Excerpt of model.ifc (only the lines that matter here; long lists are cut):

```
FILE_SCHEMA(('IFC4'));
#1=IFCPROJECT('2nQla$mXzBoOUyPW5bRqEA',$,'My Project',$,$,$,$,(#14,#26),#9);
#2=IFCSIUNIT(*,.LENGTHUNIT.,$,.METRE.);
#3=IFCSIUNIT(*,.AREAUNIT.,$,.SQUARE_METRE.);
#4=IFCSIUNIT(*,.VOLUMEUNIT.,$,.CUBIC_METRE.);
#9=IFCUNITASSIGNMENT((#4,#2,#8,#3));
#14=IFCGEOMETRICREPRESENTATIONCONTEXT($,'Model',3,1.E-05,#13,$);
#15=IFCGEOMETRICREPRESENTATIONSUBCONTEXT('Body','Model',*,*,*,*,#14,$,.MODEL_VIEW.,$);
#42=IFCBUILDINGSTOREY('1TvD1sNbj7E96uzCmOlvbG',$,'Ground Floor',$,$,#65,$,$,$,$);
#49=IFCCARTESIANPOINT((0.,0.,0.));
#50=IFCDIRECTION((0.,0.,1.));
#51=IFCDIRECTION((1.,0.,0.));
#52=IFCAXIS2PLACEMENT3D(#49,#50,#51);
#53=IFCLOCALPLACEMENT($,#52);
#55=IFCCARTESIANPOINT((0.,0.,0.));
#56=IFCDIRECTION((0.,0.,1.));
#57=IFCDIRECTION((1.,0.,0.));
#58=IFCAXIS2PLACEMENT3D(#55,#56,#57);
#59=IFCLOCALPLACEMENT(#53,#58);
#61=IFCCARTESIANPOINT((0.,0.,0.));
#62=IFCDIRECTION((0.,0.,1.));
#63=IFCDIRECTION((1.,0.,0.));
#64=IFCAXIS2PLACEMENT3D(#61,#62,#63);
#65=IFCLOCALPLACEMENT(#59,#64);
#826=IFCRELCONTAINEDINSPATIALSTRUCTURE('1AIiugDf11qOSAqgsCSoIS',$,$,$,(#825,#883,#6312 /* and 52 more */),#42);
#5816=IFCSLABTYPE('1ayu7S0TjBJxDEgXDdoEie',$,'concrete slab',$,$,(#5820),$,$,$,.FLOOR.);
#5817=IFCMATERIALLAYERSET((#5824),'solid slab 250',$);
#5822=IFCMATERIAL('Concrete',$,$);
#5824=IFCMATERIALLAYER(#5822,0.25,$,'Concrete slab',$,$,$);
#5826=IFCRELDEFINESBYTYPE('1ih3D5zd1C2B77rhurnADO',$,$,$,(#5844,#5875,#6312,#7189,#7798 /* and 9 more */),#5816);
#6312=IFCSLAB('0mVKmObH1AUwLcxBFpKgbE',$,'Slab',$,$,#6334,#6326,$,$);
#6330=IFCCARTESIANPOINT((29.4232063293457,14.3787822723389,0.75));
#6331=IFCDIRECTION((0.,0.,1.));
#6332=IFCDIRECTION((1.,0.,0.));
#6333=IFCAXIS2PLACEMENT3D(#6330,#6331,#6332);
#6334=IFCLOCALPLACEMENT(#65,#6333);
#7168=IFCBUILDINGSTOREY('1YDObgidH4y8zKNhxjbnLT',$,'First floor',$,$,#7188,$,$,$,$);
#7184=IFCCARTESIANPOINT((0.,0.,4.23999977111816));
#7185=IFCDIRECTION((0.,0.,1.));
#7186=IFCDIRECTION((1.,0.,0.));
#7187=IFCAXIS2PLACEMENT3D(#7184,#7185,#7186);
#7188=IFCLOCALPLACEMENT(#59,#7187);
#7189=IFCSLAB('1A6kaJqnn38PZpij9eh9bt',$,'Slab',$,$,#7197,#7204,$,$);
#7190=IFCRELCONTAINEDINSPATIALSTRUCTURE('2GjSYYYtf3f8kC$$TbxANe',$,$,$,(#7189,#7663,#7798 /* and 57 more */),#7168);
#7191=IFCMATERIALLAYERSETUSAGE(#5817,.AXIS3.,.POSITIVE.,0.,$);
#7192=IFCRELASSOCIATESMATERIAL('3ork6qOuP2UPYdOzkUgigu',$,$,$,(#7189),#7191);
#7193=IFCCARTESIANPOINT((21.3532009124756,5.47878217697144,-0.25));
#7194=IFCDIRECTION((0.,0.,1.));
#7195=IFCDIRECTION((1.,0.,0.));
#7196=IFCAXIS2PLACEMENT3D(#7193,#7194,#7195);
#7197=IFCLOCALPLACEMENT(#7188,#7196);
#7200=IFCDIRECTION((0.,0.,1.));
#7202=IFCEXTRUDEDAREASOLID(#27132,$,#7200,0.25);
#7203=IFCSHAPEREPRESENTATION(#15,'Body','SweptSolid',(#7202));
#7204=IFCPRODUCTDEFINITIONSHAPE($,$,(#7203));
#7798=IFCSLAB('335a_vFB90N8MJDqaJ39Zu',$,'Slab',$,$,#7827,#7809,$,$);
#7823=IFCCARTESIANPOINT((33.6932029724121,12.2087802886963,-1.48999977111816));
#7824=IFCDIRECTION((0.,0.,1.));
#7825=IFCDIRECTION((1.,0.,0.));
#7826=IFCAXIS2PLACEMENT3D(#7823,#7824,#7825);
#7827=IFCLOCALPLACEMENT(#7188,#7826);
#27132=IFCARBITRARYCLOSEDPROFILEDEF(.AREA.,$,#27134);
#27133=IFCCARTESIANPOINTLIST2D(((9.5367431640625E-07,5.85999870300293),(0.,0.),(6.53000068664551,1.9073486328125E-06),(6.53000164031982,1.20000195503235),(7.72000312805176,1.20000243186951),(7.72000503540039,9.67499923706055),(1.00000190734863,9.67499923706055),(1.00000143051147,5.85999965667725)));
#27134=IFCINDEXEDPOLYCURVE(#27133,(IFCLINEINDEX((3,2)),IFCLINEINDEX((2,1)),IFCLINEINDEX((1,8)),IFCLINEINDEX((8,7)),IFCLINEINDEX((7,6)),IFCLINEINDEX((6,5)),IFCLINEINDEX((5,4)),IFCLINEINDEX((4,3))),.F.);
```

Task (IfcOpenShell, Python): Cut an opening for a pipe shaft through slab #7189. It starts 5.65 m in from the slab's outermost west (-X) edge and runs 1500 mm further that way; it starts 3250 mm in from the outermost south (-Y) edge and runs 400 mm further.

```python
import numpy as np
import ifcopenshell
import ifcopenshell.api.feature
import ifcopenshell.api.geometry
import ifcopenshell.api.root
import ifcopenshell.geom
import ifcopenshell.util.placement
import ifcopenshell.util.representation
import ifcopenshell.util.shape
import ifcopenshell.util.unit

model = ifcopenshell.open("model.ifc")
unit_scale = ifcopenshell.util.unit.calculate_unit_scale(model)
settings = ifcopenshell.geom.settings()


def volume(element):
    """Net volume in cubic metres, openings subtracted."""
    shape = ifcopenshell.geom.create_shape(settings, element)
    return ifcopenshell.util.shape.get_volume(shape.geometry)


slab = model.by_guid("1A6kaJqnn38PZpij9eh9bt")
before = volume(slab)

# Extent in the slab's own axes, in metres. The edges named are its -X and -Y sides.
slab_shape = ifcopenshell.geom.create_shape(settings, slab)
vertices = ifcopenshell.util.shape.get_vertices(slab_shape.geometry)
x_min, y_min, bottom = vertices.min(axis=0)
top = vertices[:, 2].max()

opening = ifcopenshell.api.root.create_entity(model, ifc_class="IfcOpeningElement", name="Pipe shaft opening", predefined_type="OPENING")
context = ifcopenshell.util.representation.get_context(model, "Model", "Body", "MODEL_VIEW")
width, depth = 1.5, 0.4
outline = [(0.0, 0.0), (width, 0.0), (width, depth), (0.0, depth), (0.0, 0.0)]
# Overshoot both faces by 50 mm so the cut is clean.
shape = ifcopenshell.api.geometry.add_slab_representation(
    model, context=context, depth=top - bottom + 0.1, polyline=outline
)
ifcopenshell.api.geometry.assign_representation(model, product=opening, representation=shape)

matrix = ifcopenshell.util.placement.get_local_placement(slab.ObjectPlacement)
matrix[:, 3] = matrix @ np.append(np.array([x_min + 5.65, y_min + 3.25, bottom - 0.05]) / unit_scale, 1.0)
ifcopenshell.api.geometry.edit_object_placement(model, product=opening, matrix=matrix, is_si=False)
ifcopenshell.api.feature.add_feature(model, feature=opening, element=slab)

after = volume(slab)

print(f"slab volume {before:.3f} -> {after:.3f} m3")

model.write("model_v2.ifc")
```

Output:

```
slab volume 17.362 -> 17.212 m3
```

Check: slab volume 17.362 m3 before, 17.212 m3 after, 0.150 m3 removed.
